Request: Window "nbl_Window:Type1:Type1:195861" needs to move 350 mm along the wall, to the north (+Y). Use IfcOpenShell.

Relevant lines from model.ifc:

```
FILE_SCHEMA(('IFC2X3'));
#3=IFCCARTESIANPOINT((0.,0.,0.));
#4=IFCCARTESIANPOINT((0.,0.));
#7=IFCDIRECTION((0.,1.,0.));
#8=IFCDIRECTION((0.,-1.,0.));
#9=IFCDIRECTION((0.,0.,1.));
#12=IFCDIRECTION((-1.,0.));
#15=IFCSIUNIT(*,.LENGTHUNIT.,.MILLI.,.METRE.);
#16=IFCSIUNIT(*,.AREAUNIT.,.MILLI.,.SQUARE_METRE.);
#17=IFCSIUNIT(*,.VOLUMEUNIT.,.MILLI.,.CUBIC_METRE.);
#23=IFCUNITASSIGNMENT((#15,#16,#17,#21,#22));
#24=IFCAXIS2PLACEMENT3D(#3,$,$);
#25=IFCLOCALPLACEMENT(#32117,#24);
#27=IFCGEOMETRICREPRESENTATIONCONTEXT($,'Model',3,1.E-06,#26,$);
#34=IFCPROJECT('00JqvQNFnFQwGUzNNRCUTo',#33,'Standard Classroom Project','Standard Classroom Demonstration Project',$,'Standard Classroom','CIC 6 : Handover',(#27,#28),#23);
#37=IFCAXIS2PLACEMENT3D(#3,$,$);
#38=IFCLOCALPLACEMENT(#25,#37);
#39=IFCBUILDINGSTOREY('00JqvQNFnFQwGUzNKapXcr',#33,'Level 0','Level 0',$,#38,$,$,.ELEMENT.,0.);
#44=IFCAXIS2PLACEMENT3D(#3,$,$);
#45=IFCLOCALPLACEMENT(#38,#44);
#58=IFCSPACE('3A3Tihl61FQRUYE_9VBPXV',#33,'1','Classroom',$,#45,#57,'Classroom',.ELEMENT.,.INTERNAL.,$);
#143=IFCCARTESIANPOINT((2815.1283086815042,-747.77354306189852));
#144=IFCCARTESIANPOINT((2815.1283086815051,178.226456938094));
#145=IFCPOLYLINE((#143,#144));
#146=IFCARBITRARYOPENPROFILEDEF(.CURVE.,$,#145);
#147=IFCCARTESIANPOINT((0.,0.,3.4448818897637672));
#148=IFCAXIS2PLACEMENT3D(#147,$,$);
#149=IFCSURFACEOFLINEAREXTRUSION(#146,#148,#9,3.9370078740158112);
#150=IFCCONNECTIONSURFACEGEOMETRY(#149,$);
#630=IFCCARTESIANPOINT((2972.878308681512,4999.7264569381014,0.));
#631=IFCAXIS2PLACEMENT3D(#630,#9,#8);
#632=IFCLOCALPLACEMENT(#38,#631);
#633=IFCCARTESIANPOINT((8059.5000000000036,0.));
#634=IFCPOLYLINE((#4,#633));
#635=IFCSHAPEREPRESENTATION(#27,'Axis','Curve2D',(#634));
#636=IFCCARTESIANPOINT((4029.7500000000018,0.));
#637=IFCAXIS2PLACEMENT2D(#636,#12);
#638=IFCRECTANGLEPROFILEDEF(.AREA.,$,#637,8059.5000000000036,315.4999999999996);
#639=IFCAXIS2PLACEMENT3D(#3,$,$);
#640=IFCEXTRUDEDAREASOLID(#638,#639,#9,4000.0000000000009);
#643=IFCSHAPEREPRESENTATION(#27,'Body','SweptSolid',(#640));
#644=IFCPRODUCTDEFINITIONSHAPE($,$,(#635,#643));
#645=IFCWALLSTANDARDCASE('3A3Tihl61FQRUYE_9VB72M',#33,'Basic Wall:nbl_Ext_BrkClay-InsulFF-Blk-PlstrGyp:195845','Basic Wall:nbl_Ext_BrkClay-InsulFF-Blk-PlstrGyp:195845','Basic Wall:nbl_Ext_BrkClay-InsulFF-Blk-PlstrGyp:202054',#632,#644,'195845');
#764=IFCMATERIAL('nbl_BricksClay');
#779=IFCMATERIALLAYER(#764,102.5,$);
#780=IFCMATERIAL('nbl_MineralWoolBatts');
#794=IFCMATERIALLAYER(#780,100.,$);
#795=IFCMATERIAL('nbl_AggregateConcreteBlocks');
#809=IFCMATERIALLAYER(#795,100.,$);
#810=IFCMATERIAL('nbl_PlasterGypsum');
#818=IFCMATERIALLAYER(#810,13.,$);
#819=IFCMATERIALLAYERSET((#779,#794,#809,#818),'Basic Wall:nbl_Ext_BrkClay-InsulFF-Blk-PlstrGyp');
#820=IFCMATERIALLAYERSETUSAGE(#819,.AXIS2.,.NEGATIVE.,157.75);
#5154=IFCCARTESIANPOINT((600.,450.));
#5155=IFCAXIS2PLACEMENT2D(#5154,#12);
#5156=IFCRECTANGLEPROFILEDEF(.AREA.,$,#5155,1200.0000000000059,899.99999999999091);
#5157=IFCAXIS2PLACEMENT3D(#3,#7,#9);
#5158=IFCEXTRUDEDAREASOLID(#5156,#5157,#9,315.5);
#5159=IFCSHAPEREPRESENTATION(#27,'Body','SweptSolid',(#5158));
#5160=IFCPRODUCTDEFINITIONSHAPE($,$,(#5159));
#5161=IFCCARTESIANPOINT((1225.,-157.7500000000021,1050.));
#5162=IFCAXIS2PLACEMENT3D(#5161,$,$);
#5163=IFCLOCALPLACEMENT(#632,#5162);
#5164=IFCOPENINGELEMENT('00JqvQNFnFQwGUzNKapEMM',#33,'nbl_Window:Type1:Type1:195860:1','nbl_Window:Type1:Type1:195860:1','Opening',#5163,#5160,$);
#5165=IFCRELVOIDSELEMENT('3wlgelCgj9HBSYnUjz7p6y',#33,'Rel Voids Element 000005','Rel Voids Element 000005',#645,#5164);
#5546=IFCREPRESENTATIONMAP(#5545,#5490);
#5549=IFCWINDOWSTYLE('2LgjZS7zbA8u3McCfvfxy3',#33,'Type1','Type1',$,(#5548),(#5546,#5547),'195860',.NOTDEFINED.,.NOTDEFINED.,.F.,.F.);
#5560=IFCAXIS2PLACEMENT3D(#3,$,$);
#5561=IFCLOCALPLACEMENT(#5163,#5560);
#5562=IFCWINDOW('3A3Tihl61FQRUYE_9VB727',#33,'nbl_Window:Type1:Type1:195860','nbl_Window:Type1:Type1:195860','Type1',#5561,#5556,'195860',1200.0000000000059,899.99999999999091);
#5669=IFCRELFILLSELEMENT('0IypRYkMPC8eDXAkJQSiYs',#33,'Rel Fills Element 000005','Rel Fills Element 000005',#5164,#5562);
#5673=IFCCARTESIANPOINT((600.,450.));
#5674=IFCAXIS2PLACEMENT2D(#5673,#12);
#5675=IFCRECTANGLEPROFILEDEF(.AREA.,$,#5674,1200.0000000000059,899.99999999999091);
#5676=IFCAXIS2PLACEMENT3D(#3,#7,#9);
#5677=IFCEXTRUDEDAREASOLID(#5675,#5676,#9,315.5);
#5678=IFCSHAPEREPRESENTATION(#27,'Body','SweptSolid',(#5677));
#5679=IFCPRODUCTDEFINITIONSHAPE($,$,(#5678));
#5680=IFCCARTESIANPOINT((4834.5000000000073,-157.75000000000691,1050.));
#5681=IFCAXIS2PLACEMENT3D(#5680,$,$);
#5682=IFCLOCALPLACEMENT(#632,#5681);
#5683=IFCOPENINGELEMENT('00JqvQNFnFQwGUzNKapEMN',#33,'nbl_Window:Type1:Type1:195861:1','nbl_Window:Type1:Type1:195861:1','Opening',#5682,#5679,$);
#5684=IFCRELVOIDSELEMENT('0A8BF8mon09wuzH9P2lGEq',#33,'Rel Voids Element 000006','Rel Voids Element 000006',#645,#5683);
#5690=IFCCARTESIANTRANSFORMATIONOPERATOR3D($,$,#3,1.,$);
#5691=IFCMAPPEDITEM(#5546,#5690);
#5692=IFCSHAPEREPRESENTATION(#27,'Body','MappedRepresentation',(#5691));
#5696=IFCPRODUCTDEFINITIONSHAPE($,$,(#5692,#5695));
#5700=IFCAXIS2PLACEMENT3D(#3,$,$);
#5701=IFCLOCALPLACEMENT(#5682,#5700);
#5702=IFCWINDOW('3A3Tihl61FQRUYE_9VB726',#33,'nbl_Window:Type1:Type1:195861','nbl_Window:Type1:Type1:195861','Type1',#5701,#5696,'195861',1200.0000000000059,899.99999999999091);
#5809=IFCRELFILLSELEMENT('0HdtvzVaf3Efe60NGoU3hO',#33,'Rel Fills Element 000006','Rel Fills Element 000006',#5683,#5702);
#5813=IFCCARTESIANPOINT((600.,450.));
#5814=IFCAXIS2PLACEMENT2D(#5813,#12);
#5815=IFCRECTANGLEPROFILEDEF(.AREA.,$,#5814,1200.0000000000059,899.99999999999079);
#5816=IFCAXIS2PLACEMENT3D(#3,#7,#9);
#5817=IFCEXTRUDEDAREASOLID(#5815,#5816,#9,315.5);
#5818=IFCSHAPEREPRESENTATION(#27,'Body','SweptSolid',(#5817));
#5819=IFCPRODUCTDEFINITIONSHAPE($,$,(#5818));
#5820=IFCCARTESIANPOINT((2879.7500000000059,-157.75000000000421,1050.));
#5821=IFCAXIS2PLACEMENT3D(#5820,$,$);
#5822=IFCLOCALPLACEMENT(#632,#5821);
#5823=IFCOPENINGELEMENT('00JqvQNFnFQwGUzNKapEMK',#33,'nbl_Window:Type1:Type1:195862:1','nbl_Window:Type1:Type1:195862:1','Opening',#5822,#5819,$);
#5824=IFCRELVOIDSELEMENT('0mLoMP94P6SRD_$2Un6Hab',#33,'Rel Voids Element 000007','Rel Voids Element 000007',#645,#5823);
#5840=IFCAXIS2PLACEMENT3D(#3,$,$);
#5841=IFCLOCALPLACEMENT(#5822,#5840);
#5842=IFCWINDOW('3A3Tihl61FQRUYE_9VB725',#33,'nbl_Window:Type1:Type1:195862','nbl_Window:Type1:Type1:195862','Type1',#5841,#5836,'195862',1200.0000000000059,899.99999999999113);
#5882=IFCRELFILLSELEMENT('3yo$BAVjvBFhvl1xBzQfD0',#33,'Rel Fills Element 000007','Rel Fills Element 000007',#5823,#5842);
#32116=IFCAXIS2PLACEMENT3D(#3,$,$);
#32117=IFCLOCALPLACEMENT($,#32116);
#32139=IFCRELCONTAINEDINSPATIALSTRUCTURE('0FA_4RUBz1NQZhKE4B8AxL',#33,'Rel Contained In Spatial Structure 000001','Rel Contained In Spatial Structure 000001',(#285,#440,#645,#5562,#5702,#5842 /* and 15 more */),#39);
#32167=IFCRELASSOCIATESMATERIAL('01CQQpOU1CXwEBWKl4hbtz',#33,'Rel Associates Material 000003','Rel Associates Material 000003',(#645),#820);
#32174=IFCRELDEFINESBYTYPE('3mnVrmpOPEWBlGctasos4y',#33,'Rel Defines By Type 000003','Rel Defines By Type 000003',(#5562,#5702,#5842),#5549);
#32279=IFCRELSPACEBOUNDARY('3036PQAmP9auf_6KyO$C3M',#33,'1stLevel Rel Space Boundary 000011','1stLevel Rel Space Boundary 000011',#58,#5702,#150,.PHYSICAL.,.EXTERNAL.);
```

```python
import numpy as np
import ifcopenshell
import ifcopenshell.api.geometry
import ifcopenshell.util.placement
import ifcopenshell.util.unit

model = ifcopenshell.open("model.ifc")
unit_scale = ifcopenshell.util.unit.calculate_unit_scale(model)

window = model.by_id(5702)
opening = window.FillsVoids[0].RelatingOpeningElement
wall = opening.VoidsElements[0].RelatingBuildingElement

wall_matrix = ifcopenshell.util.placement.get_local_placement(wall.ObjectPlacement)
shift = wall_matrix[:3, 0] * -0.35 / unit_scale
before = ifcopenshell.util.placement.get_local_placement(window.ObjectPlacement)[:3, 3].copy()

# The window is placed relative to its opening, so it follows when the opening moves.
matrix = ifcopenshell.util.placement.get_local_placement(opening.ObjectPlacement)
matrix[:3, 3] += shift
ifcopenshell.api.geometry.edit_object_placement(
    model, product=opening, matrix=matrix, is_si=False, should_transform_children=True
)

# Space boundary surfaces are stored in each space's coordinates; move them too.
for rel in window.ProvidesBoundaries:
    if not rel.ConnectionGeometry:
        continue
    surface = rel.ConnectionGeometry.SurfaceOnRelatingElement
    space_matrix = ifcopenshell.util.placement.get_local_placement(rel.RelatingSpace.ObjectPlacement)
    point = np.array(surface.Position.Location.Coordinates) + space_matrix[:3, :3].T @ shift
    surface.Position = model.createIfcAxis2Placement3D(
        model.createIfcCartesianPoint(point.tolist()), surface.Position.Axis, surface.Position.RefDirection
    )

after = ifcopenshell.util.placement.get_local_placement(window.ObjectPlacement)[:3, 3]
print("window moved by", (after - before).round(3) + 0.0)

model.write("model_edited.ifc")
```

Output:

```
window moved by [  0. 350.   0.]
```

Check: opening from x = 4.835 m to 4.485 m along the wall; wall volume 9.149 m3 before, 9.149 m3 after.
